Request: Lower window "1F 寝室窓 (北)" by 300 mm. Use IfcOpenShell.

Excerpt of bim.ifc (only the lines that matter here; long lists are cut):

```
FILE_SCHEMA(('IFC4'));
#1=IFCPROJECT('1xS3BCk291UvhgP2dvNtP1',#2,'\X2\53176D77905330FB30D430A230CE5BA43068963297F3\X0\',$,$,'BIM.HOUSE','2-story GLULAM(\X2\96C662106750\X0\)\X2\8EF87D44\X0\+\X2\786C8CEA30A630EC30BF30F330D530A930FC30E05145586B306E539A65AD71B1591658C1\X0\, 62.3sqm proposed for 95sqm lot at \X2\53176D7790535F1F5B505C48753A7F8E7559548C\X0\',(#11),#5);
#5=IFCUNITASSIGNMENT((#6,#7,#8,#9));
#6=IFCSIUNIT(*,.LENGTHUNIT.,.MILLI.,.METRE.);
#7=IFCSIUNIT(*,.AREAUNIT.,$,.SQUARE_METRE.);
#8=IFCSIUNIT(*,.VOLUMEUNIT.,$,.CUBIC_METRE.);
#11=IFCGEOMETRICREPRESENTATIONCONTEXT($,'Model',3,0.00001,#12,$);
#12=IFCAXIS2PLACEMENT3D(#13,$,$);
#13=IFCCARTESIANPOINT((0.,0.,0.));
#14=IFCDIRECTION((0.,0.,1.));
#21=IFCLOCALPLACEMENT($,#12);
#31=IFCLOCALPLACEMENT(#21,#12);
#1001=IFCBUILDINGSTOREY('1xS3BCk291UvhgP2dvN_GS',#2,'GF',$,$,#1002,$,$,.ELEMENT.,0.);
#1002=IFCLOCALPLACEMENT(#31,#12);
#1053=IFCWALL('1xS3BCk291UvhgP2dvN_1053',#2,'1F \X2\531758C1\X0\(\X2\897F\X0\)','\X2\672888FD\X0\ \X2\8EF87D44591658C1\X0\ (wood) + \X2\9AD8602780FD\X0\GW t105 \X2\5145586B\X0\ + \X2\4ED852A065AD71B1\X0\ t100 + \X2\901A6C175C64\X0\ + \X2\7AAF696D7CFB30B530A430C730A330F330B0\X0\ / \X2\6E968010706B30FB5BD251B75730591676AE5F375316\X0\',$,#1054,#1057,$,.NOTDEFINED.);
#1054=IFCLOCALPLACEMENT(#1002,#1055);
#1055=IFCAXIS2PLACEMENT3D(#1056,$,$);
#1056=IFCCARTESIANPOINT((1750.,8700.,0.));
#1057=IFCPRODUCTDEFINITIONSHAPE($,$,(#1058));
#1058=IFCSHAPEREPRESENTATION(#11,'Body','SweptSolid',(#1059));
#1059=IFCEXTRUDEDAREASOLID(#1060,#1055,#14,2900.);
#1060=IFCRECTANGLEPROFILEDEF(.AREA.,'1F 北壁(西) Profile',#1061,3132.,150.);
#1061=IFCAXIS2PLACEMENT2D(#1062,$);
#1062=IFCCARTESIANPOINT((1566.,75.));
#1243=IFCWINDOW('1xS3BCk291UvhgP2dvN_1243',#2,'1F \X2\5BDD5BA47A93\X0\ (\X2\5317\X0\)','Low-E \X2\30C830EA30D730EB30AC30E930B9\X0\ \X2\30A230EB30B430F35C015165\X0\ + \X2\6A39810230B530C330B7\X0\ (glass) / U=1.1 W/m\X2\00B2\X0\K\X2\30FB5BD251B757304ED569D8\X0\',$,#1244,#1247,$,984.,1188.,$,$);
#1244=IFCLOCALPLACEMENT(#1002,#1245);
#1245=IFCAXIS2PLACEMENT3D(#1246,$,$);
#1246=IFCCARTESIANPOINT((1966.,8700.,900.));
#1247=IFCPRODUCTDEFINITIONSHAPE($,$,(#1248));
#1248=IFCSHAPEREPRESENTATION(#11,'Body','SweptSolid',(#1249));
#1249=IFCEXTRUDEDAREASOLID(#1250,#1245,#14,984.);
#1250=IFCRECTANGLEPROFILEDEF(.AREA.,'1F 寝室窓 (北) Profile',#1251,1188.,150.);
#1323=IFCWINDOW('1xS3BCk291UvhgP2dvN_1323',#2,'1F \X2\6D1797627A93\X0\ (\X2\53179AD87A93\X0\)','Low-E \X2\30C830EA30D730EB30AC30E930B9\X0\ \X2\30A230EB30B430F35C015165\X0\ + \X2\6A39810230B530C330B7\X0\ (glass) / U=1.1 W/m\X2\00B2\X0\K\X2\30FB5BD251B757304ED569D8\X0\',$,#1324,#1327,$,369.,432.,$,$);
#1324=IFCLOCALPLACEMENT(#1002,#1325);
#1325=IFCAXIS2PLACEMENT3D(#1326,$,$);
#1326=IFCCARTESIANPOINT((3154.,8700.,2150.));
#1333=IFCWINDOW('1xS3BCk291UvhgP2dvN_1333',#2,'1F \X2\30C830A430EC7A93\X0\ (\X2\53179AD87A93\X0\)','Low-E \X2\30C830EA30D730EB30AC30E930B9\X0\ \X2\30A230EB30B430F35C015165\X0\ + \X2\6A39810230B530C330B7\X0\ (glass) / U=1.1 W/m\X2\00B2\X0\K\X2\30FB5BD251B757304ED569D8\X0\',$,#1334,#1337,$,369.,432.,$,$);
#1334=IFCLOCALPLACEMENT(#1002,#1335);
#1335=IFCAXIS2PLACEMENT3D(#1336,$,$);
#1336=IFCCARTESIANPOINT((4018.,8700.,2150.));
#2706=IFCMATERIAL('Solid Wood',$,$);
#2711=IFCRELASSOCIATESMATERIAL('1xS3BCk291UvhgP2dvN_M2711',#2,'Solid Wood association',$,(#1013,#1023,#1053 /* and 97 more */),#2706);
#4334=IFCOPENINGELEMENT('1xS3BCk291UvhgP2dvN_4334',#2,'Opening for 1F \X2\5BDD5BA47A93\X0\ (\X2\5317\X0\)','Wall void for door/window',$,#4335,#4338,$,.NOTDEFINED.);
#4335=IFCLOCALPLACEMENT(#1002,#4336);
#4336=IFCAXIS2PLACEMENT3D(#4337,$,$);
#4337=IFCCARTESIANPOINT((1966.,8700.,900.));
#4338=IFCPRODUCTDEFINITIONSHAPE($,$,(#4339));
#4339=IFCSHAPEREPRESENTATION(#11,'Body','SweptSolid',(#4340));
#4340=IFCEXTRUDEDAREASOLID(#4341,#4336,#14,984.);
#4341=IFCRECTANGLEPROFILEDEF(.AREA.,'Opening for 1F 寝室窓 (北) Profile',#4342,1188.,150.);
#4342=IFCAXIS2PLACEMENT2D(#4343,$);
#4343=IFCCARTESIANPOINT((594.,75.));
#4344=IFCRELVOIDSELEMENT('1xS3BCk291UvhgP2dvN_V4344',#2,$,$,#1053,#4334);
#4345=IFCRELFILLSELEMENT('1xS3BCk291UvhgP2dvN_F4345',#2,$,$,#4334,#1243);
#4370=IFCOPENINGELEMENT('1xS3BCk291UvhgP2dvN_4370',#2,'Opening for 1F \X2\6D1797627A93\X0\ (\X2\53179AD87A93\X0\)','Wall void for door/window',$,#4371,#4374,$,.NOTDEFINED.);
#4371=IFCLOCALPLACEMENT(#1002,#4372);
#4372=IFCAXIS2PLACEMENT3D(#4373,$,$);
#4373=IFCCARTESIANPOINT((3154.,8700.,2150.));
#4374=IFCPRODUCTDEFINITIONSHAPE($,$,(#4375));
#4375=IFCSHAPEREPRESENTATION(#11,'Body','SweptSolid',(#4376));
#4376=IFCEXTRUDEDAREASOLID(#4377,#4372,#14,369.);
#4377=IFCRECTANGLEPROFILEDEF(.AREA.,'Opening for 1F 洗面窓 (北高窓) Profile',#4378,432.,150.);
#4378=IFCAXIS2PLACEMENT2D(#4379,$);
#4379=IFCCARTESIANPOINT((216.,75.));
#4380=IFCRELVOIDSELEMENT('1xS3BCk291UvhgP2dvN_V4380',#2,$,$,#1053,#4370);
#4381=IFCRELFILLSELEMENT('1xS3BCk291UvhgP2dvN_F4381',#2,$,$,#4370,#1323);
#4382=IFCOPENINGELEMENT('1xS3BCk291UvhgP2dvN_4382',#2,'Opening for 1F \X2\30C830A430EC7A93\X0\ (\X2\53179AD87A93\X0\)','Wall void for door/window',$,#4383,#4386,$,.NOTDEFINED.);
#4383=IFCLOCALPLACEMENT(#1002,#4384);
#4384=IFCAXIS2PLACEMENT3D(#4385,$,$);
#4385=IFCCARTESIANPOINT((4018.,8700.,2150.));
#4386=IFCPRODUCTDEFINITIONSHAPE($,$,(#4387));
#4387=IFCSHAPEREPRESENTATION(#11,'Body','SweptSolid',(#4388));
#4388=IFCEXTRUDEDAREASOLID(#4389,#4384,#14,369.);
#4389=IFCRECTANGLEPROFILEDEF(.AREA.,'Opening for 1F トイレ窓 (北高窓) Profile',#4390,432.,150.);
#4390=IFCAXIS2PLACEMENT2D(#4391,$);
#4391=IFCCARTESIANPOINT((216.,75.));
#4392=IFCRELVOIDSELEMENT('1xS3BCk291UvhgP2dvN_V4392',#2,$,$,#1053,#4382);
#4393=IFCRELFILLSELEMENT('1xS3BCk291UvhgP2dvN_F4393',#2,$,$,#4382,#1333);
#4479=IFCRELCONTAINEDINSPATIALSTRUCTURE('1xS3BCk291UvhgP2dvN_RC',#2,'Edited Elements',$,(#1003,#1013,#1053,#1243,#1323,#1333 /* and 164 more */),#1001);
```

```python
import numpy as np
import ifcopenshell
import ifcopenshell.api.geometry
import ifcopenshell.util.placement
import ifcopenshell.util.unit

model = ifcopenshell.open("bim.ifc")
unit_scale = ifcopenshell.util.unit.calculate_unit_scale(model)

window = model.by_id(1243)
opening = window.FillsVoids[0].RelatingOpeningElement
dz = -0.3 / unit_scale

shift = np.array([0.0, 0.0, dz])
# The window is not placed relative to its opening, so move both.
for product in (opening, window):
    matrix = ifcopenshell.util.placement.get_local_placement(product.ObjectPlacement)
    matrix[:3, 3] += shift
    ifcopenshell.api.geometry.edit_object_placement(model, product=product, matrix=matrix, is_si=False)

print(f"moved by {dz * unit_scale:+.3f} m")

model.write("bim_rev.ifc")
```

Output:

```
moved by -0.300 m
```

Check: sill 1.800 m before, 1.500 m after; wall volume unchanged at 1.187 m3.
